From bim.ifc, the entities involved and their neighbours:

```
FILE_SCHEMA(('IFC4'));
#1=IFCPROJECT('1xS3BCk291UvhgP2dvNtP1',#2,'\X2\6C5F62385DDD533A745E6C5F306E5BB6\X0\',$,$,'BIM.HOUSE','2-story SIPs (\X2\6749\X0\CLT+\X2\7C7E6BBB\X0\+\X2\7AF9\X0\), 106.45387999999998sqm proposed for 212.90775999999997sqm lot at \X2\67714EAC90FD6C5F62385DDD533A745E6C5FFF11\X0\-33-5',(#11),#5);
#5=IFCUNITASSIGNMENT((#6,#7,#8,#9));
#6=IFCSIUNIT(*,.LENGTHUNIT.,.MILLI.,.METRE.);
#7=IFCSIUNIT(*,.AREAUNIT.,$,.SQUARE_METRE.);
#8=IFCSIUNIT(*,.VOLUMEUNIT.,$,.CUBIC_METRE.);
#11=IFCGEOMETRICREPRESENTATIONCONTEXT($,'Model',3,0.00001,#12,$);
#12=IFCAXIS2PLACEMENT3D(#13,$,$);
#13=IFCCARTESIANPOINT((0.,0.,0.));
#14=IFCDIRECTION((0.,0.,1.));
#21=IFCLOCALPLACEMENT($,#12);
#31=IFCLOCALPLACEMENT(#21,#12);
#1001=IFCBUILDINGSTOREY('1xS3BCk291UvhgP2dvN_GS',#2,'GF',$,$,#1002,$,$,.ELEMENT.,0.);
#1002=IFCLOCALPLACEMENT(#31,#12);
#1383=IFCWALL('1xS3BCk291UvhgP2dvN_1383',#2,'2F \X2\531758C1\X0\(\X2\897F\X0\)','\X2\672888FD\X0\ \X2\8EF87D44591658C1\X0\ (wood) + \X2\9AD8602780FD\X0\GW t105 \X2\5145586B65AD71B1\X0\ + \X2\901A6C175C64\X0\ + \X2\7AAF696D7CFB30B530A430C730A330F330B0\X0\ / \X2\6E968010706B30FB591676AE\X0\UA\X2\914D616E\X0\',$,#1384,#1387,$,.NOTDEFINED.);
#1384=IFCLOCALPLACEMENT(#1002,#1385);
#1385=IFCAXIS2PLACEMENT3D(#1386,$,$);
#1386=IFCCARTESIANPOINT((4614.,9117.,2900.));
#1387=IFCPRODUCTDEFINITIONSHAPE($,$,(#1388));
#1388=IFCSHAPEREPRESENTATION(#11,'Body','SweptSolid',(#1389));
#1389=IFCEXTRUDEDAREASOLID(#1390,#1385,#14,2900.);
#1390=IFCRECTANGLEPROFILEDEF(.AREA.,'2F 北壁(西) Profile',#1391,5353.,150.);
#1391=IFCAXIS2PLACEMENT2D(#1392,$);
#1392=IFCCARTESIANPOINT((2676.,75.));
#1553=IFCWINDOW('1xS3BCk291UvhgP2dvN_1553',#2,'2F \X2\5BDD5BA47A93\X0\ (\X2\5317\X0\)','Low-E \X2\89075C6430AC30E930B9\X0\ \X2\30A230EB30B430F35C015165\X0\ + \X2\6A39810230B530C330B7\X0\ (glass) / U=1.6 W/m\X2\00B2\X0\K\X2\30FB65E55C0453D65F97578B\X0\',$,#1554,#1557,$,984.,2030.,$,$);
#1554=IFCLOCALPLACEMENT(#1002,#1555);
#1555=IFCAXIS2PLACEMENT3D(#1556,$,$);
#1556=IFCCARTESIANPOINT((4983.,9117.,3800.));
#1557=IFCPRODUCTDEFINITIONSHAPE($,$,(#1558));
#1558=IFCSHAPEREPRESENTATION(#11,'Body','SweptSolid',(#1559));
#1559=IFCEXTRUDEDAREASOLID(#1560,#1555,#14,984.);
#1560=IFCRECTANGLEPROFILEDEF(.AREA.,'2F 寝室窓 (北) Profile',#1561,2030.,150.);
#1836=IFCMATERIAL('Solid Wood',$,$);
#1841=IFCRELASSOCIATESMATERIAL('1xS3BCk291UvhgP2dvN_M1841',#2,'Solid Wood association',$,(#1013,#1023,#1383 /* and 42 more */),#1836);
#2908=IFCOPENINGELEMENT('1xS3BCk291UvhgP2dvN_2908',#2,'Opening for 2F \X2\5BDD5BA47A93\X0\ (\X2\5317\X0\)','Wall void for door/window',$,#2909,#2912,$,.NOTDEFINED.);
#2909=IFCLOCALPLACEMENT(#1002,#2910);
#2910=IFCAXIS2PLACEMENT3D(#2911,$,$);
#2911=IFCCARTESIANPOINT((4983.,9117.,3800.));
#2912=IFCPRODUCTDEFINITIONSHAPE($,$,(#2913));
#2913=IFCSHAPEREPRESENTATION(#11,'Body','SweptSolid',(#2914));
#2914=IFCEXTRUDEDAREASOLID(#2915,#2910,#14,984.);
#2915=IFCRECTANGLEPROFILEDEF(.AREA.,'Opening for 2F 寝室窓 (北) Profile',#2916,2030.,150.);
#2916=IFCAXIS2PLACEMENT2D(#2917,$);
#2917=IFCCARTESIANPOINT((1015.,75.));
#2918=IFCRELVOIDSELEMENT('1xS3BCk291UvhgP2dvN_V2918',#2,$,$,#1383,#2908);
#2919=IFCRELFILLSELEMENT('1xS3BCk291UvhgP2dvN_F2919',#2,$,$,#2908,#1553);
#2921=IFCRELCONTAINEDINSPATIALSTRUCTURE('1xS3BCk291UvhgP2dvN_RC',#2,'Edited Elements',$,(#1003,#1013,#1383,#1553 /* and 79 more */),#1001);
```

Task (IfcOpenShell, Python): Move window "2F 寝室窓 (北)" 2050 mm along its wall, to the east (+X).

```python
import ifcopenshell
import ifcopenshell.api.geometry
import ifcopenshell.util.placement
import ifcopenshell.util.unit

model = ifcopenshell.open("bim.ifc")
unit_scale = ifcopenshell.util.unit.calculate_unit_scale(model)

window = model.by_guid("1xS3BCk291UvhgP2dvN_1553")
opening = window.FillsVoids[0].RelatingOpeningElement
wall = opening.VoidsElements[0].RelatingBuildingElement

wall_matrix = ifcopenshell.util.placement.get_local_placement(wall.ObjectPlacement)
shift = wall_matrix[:3, 0] * 2.05 / unit_scale
before = ifcopenshell.util.placement.get_local_placement(window.ObjectPlacement)[:3, 3].copy()

# The window is not placed relative to its opening, so move both.
for product in (opening, window):
    matrix = ifcopenshell.util.placement.get_local_placement(product.ObjectPlacement)
    matrix[:3, 3] += shift
    ifcopenshell.api.geometry.edit_object_placement(model, product=product, matrix=matrix, is_si=False)

after = ifcopenshell.util.placement.get_local_placement(window.ObjectPlacement)[:3, 3]
print("window moved by", (after - before).round(3) + 0.0)

model.write("bim_v2.ifc")
```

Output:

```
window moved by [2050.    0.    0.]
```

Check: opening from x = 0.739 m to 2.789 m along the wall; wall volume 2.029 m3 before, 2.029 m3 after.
